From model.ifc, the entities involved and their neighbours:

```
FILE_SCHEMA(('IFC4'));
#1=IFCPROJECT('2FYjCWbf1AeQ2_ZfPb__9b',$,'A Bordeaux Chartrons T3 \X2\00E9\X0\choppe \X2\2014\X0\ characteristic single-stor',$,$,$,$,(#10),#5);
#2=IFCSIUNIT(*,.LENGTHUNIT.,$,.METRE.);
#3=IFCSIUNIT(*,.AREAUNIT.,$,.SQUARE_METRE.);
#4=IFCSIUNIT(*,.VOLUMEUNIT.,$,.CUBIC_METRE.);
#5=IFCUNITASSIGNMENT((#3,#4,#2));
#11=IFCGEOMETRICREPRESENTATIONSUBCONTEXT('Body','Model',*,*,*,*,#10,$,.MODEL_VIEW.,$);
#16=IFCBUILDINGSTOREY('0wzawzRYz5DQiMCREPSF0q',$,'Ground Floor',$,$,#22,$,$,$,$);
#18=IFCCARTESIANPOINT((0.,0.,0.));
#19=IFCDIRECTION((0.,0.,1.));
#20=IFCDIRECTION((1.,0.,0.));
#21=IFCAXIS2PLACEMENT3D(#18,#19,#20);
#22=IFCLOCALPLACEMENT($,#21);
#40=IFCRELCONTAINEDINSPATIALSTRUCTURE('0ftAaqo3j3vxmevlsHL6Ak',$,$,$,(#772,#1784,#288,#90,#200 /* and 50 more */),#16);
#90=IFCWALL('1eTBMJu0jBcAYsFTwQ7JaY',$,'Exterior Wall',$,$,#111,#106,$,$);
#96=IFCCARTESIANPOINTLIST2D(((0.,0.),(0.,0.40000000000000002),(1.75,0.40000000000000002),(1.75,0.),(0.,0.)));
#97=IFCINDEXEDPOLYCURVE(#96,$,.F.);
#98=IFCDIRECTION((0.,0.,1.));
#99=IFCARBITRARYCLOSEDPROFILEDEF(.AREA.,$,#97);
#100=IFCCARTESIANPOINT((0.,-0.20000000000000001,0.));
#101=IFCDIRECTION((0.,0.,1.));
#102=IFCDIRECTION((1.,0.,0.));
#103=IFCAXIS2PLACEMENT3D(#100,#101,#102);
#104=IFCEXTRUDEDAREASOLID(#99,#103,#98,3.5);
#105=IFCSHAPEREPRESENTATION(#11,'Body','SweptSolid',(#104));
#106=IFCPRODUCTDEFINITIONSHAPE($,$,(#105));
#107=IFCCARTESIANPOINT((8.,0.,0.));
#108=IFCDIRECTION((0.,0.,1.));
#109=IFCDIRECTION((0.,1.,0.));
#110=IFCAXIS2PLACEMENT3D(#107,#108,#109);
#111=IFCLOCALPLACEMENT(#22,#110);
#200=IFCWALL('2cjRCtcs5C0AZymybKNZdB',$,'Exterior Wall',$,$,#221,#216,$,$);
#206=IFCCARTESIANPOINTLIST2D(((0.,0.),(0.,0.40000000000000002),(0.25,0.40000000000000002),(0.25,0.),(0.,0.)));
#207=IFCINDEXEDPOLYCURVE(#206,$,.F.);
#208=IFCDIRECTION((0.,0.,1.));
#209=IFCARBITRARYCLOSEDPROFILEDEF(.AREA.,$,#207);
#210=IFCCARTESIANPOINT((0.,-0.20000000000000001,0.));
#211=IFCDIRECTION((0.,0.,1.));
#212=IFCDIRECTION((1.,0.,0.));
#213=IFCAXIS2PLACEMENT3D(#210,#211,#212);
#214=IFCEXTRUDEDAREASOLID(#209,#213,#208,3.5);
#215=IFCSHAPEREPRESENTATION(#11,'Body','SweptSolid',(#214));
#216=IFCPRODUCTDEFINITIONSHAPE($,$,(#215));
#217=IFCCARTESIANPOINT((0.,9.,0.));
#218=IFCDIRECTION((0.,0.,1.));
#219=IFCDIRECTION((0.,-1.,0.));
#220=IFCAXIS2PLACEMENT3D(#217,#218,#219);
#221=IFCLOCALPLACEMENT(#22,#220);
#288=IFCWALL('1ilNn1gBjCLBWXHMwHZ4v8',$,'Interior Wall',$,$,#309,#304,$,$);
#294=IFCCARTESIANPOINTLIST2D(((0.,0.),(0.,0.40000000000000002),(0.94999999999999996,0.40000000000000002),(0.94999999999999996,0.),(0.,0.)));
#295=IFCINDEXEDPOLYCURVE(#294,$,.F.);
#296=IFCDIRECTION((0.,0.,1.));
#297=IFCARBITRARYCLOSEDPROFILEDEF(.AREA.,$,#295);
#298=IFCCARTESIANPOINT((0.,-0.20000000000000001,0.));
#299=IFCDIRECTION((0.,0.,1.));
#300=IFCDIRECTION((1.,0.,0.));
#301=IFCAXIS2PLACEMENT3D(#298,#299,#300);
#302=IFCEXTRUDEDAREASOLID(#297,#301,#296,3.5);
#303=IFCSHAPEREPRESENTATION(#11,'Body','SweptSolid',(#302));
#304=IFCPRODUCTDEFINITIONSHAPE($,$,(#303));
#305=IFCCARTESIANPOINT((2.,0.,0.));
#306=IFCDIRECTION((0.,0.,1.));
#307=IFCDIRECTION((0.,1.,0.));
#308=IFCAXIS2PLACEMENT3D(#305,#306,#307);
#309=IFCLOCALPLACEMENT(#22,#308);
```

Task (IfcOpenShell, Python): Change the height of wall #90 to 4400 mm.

```python
import ifcopenshell
import ifcopenshell.geom
import ifcopenshell.util.representation
import ifcopenshell.util.shape

model = ifcopenshell.open("model.ifc")
settings = ifcopenshell.geom.settings()


def volume(element):
    """Net volume in cubic metres, openings subtracted."""
    shape = ifcopenshell.geom.create_shape(settings, element)
    return ifcopenshell.util.shape.get_volume(shape.geometry)


wall = model.by_id(90)
before = volume(wall)

body = ifcopenshell.util.representation.get_representation(wall, "Model", "Body")
solid = body.Items[0]
old_height = solid.Depth
solid.Depth = 4.4
after = volume(wall)

print(f"height {old_height:g} -> {solid.Depth:g}, volume {before:.3f} -> {after:.3f} m3")

model.write("model_updated.ifc")
```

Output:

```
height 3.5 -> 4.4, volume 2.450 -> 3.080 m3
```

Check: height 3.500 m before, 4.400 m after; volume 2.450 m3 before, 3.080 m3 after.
